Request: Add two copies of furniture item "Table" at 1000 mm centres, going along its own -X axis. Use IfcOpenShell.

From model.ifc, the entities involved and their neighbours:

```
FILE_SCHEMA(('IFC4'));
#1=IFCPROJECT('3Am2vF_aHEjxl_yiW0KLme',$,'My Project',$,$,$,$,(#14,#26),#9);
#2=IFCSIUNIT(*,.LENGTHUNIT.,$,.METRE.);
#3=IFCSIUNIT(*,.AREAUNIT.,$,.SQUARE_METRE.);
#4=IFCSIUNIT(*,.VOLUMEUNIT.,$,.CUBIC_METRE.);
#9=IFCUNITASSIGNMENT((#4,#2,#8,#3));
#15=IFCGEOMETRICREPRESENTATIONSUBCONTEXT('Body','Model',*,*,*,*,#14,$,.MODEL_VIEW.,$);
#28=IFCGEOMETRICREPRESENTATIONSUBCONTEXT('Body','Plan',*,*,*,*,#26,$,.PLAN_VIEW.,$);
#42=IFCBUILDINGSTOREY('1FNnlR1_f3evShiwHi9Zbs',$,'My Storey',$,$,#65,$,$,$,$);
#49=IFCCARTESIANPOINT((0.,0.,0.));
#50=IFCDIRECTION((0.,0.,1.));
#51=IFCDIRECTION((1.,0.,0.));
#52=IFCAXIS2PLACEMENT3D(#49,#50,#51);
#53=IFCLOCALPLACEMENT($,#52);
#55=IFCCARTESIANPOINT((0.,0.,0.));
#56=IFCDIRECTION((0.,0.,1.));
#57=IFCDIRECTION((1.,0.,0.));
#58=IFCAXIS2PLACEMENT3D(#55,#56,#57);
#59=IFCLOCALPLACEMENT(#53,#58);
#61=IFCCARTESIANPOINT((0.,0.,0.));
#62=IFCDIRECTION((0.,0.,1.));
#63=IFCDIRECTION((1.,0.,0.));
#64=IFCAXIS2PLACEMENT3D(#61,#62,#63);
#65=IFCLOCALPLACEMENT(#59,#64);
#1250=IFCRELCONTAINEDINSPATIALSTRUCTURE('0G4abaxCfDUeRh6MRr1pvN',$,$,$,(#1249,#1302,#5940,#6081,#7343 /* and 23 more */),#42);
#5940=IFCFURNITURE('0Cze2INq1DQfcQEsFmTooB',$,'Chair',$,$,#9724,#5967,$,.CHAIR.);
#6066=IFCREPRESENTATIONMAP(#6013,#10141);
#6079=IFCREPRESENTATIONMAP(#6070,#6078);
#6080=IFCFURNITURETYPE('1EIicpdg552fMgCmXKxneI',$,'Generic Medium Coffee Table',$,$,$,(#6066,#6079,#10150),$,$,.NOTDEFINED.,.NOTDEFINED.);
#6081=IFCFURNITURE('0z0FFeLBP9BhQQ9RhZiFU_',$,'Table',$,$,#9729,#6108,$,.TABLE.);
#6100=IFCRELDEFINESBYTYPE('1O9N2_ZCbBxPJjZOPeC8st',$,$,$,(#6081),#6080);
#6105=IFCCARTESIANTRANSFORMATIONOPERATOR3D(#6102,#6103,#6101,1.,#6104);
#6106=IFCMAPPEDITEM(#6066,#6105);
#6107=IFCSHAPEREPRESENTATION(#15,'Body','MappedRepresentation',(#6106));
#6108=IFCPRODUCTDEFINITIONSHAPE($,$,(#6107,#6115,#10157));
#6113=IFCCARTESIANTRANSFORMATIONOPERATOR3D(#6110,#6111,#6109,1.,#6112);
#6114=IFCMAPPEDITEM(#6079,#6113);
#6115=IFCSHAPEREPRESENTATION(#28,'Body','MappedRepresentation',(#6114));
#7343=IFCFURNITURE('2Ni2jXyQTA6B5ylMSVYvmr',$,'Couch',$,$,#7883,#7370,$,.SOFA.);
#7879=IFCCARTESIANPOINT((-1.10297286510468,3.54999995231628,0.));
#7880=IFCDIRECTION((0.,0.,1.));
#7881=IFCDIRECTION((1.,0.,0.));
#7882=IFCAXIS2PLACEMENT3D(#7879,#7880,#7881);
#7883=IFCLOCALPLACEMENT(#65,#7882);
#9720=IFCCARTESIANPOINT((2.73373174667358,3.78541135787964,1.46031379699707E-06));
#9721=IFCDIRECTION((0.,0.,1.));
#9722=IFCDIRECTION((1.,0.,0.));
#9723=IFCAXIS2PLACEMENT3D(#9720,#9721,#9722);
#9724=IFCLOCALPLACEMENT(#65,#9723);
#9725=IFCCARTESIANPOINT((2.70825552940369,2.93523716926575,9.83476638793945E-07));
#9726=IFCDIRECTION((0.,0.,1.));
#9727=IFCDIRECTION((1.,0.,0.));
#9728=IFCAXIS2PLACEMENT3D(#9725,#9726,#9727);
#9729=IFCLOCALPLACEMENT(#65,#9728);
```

```python
import ifcopenshell
import ifcopenshell.api.geometry
import ifcopenshell.api.root
import ifcopenshell.util.element
import ifcopenshell.util.placement
import ifcopenshell.util.unit

model = ifcopenshell.open("model.ifc")
unit_scale = ifcopenshell.util.unit.calculate_unit_scale(model)

source = model.by_guid("0z0FFeLBP9BhQQ9RhZiFU_")
base = ifcopenshell.util.placement.get_local_placement(source.ObjectPlacement)
step = -base[:3, 0] * 1 / unit_scale

for i in range(1, 3):
    copy = ifcopenshell.api.root.copy_class(model, product=source)
    copy.Representation = ifcopenshell.util.element.copy_deep(
        model, source.Representation, exclude=["IfcGeometricRepresentationContext", "IfcRepresentationMap"]
    )
    matrix = base.copy()
    matrix[:3, 3] += i * step
    print("added at", matrix[:3, 3].round(3) + 0.0)
    ifcopenshell.api.geometry.edit_object_placement(model, product=copy, matrix=matrix, is_si=False)

model.write("model-out.ifc")
```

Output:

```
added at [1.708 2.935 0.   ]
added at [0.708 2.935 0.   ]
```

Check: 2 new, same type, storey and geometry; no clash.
